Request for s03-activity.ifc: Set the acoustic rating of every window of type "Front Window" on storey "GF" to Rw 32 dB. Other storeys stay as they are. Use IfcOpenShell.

First a look at what the model holds.

```python
import ifcopenshell
import ifcopenshell.util.element

model = ifcopenshell.open("s03-activity.ifc")
print(model.schema)
storey = next(s for s in model.by_type("IfcBuildingStorey") if s.Name == "GF")
windows = [e for e in ifcopenshell.util.element.get_decomposition(storey) if e.is_a("IfcWindow")]
seen = {}
for e in windows:
    element_type = ifcopenshell.util.element.get_type(e)
    key = (element_type.Name if element_type != e and element_type else None, ifcopenshell.util.element.get_pset(e, "Pset_WindowCommon", "AcousticRating"))
    seen[key] = seen.get(key, 0) + 1
for (name, value), count in sorted(seen.items(), key=str):
    print(count, "x", name, "|", value)
```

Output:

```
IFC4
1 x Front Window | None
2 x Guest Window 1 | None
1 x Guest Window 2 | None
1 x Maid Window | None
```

```python
import ifcopenshell
import ifcopenshell.api.pset
import ifcopenshell.util.element

model = ifcopenshell.open("s03-activity.ifc")

storey = next(s for s in model.by_type("IfcBuildingStorey") if s.Name == "GF")
windows = [e for e in ifcopenshell.util.element.get_decomposition(storey) if e.is_a("IfcWindow")]

count = 0
for e in windows:
    element_type = ifcopenshell.util.element.get_type(e)
    if element_type in (None, e) or element_type.Name != "Front Window":
        continue
    # add_pset returns the element's existing set when there is one.
    pset = ifcopenshell.api.pset.add_pset(model, product=e, name="Pset_WindowCommon")
    ifcopenshell.api.pset.edit_pset(model, pset=pset, properties={"AcousticRating": "Rw 32 dB"})
    count += 1

print(count, "windows updated")

model.write("s03-activity_rev.ifc")
```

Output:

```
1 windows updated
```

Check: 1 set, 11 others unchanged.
